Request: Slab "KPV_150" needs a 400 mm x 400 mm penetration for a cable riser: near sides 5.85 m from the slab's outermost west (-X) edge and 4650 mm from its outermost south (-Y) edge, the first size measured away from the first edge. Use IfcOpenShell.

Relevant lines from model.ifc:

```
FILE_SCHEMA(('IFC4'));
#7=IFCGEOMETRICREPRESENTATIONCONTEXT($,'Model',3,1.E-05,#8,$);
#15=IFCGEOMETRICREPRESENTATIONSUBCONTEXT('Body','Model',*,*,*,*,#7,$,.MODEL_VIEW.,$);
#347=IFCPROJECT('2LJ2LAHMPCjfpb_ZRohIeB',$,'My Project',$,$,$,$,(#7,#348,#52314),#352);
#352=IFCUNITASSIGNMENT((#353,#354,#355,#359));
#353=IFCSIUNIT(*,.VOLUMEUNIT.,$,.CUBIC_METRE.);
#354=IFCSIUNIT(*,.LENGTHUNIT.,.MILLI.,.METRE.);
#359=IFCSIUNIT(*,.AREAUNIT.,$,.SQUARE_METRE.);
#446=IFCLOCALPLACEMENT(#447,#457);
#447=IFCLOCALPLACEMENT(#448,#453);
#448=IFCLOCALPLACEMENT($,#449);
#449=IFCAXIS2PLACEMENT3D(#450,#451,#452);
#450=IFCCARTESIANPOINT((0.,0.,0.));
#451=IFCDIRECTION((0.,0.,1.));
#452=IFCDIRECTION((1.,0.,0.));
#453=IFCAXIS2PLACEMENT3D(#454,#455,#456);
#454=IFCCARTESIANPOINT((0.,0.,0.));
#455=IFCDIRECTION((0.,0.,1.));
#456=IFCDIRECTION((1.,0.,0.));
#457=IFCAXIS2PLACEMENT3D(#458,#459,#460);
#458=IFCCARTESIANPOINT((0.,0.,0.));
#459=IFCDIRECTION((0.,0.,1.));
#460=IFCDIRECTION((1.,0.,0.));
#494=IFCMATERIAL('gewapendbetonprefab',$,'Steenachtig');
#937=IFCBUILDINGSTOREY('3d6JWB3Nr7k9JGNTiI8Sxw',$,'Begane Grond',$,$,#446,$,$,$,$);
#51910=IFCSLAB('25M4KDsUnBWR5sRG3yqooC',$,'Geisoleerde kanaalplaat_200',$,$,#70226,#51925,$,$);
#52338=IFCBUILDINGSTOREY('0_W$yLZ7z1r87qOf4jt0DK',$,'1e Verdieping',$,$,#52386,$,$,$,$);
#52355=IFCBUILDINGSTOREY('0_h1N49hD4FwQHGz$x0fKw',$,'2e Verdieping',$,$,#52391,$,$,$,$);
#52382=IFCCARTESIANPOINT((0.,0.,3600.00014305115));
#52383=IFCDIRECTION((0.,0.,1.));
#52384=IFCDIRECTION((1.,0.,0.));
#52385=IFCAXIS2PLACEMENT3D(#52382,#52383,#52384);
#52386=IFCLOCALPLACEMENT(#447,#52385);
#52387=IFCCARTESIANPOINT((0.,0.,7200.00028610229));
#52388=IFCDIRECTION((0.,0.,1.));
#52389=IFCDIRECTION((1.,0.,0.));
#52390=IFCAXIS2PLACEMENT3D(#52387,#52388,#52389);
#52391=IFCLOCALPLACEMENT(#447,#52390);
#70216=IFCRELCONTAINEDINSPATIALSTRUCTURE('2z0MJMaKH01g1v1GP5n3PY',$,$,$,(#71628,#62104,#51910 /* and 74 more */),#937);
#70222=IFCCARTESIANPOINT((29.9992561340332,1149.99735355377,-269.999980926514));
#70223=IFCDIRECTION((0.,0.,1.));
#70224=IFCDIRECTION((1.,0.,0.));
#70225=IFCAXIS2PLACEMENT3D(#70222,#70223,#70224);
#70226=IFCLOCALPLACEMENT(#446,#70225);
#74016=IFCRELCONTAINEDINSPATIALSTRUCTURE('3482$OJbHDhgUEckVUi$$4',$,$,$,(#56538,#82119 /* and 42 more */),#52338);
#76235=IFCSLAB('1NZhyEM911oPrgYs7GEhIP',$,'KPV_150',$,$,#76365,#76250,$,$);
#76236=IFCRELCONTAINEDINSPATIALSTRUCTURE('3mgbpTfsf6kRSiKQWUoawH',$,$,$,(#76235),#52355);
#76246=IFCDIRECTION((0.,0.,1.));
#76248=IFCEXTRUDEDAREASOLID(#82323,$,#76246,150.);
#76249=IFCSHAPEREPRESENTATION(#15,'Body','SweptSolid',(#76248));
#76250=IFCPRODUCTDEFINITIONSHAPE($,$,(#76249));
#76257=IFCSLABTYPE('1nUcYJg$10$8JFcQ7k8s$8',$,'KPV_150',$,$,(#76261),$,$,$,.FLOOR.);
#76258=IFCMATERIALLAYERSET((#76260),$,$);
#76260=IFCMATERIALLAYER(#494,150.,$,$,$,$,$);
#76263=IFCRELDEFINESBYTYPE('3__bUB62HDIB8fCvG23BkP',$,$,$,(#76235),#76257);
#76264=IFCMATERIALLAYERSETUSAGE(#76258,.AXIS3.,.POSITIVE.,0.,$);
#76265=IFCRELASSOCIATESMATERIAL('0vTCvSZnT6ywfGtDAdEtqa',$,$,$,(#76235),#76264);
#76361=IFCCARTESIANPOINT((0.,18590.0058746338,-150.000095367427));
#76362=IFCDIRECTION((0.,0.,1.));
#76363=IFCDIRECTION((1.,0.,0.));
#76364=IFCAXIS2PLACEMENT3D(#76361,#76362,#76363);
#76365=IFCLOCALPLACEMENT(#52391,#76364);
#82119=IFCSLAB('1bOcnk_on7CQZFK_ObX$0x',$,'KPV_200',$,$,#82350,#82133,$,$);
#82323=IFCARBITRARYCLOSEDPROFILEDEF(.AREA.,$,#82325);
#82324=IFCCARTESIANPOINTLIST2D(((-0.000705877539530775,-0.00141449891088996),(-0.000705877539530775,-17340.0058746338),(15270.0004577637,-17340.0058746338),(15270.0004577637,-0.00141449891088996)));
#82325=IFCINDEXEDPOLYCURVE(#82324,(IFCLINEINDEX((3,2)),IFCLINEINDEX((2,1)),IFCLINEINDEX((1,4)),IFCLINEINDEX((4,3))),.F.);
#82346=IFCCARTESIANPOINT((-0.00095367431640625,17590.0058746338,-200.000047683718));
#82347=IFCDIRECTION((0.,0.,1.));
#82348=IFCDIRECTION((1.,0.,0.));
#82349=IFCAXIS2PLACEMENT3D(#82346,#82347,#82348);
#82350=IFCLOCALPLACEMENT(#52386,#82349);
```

```python
import numpy as np
import ifcopenshell
import ifcopenshell.api.feature
import ifcopenshell.api.geometry
import ifcopenshell.api.root
import ifcopenshell.geom
import ifcopenshell.util.placement
import ifcopenshell.util.representation
import ifcopenshell.util.shape
import ifcopenshell.util.unit

model = ifcopenshell.open("model.ifc")
unit_scale = ifcopenshell.util.unit.calculate_unit_scale(model)
settings = ifcopenshell.geom.settings()


def volume(element):
    """Net volume in cubic metres, openings subtracted."""
    shape = ifcopenshell.geom.create_shape(settings, element)
    return ifcopenshell.util.shape.get_volume(shape.geometry)


slab = model.by_id(76235)
before = volume(slab)

# Extent in the slab's own axes, in metres. The edges named are its -X and -Y sides.
slab_shape = ifcopenshell.geom.create_shape(settings, slab)
vertices = ifcopenshell.util.shape.get_vertices(slab_shape.geometry)
x_min, y_min, bottom = vertices.min(axis=0)
top = vertices[:, 2].max()

opening = ifcopenshell.api.root.create_entity(model, ifc_class="IfcOpeningElement", name="Cable riser opening", predefined_type="OPENING")
context = ifcopenshell.util.representation.get_context(model, "Model", "Body", "MODEL_VIEW")
width, depth = 0.4, 0.4
outline = [(0.0, 0.0), (width, 0.0), (width, depth), (0.0, depth), (0.0, 0.0)]
# Overshoot both faces by 50 mm so the cut is clean.
shape = ifcopenshell.api.geometry.add_slab_representation(
    model, context=context, depth=top - bottom + 0.1, polyline=outline
)
ifcopenshell.api.geometry.assign_representation(model, product=opening, representation=shape)

matrix = ifcopenshell.util.placement.get_local_placement(slab.ObjectPlacement)
matrix[:, 3] = matrix @ np.append(np.array([x_min + 5.85, y_min + 4.65, bottom - 0.05]) / unit_scale, 1.0)
ifcopenshell.api.geometry.edit_object_placement(model, product=opening, matrix=matrix, is_si=False)
ifcopenshell.api.feature.add_feature(model, feature=opening, element=slab)

after = volume(slab)

print(f"slab volume {before:.3f} -> {after:.3f} m3")

model.write("model_updated.ifc")
```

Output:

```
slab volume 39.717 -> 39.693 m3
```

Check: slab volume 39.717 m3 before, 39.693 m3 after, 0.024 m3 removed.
